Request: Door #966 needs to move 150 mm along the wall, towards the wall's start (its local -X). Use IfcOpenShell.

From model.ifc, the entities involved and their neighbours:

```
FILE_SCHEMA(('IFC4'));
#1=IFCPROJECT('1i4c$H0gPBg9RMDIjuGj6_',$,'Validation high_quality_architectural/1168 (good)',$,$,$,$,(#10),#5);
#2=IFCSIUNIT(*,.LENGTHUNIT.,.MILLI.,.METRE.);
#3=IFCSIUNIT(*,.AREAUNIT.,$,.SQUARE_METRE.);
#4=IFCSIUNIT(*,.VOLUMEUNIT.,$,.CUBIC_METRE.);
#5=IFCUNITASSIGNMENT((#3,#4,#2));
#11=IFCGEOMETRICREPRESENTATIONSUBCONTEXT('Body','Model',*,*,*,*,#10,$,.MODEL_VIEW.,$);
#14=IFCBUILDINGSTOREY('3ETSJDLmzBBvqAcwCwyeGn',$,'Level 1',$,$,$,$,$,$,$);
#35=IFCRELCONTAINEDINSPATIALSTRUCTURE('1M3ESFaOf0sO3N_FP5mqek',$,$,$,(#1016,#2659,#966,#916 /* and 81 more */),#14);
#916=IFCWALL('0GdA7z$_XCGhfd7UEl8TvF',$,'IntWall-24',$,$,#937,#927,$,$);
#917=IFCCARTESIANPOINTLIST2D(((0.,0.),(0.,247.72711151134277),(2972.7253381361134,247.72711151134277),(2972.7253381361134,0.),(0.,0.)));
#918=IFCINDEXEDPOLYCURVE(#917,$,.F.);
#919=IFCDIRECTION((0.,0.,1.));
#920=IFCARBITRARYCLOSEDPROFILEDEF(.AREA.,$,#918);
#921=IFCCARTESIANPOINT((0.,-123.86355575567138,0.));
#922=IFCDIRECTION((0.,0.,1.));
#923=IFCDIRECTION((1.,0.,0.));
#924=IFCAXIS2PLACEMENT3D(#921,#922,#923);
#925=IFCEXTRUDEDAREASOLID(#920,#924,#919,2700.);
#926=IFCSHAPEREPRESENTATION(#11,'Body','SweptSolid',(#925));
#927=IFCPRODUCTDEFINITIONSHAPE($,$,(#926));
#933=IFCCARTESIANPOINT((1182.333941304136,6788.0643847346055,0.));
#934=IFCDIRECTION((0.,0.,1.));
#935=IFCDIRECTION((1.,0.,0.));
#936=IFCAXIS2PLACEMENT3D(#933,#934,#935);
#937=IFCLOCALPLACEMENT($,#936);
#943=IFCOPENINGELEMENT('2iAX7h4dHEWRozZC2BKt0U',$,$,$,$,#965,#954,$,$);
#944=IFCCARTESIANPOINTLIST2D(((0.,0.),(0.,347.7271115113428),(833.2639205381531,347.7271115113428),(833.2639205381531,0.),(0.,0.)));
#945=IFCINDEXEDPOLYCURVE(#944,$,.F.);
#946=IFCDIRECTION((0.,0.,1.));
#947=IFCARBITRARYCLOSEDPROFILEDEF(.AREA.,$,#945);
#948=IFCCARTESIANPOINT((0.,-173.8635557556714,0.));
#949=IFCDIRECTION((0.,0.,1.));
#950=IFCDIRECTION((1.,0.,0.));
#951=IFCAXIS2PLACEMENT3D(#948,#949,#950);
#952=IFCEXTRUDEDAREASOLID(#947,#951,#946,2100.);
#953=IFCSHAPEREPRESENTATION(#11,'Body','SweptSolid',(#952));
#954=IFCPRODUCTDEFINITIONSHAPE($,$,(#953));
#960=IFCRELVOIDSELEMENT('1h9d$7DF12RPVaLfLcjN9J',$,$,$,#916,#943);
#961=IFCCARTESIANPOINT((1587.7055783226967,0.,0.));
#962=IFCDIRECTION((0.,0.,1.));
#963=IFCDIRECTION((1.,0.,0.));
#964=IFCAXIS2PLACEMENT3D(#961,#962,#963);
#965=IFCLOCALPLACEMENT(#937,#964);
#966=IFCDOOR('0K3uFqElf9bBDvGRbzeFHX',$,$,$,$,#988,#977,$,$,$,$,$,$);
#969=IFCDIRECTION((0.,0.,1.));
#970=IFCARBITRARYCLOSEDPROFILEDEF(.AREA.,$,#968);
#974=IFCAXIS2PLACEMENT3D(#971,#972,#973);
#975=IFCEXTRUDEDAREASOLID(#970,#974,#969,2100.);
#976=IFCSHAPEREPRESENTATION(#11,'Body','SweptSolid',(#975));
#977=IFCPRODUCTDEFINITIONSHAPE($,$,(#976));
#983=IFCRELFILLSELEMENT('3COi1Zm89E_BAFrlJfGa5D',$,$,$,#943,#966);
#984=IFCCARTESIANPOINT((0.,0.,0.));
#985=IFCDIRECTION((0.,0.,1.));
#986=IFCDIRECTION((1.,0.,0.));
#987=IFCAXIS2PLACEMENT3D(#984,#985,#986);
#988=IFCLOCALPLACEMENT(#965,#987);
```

```python
import ifcopenshell
import ifcopenshell.api.geometry
import ifcopenshell.util.placement

model = ifcopenshell.open("model.ifc")

door = model.by_guid("0K3uFqElf9bBDvGRbzeFHX")
opening = door.FillsVoids[0].RelatingOpeningElement
wall = opening.VoidsElements[0].RelatingBuildingElement

wall_matrix = ifcopenshell.util.placement.get_local_placement(wall.ObjectPlacement)
shift = wall_matrix[:3, 0] * -150.0
before = ifcopenshell.util.placement.get_local_placement(door.ObjectPlacement)[:3, 3].copy()

# The door is placed relative to its opening, so it follows when the opening moves.
matrix = ifcopenshell.util.placement.get_local_placement(opening.ObjectPlacement)
matrix[:3, 3] += shift
ifcopenshell.api.geometry.edit_object_placement(
    model, product=opening, matrix=matrix, is_si=False, should_transform_children=True
)

after = ifcopenshell.util.placement.get_local_placement(door.ObjectPlacement)[:3, 3]
print("door moved by", (after - before).round(3) + 0.0)

model.write("model-out.ifc")
```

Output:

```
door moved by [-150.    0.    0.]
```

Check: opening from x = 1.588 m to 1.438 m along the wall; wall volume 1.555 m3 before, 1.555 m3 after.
